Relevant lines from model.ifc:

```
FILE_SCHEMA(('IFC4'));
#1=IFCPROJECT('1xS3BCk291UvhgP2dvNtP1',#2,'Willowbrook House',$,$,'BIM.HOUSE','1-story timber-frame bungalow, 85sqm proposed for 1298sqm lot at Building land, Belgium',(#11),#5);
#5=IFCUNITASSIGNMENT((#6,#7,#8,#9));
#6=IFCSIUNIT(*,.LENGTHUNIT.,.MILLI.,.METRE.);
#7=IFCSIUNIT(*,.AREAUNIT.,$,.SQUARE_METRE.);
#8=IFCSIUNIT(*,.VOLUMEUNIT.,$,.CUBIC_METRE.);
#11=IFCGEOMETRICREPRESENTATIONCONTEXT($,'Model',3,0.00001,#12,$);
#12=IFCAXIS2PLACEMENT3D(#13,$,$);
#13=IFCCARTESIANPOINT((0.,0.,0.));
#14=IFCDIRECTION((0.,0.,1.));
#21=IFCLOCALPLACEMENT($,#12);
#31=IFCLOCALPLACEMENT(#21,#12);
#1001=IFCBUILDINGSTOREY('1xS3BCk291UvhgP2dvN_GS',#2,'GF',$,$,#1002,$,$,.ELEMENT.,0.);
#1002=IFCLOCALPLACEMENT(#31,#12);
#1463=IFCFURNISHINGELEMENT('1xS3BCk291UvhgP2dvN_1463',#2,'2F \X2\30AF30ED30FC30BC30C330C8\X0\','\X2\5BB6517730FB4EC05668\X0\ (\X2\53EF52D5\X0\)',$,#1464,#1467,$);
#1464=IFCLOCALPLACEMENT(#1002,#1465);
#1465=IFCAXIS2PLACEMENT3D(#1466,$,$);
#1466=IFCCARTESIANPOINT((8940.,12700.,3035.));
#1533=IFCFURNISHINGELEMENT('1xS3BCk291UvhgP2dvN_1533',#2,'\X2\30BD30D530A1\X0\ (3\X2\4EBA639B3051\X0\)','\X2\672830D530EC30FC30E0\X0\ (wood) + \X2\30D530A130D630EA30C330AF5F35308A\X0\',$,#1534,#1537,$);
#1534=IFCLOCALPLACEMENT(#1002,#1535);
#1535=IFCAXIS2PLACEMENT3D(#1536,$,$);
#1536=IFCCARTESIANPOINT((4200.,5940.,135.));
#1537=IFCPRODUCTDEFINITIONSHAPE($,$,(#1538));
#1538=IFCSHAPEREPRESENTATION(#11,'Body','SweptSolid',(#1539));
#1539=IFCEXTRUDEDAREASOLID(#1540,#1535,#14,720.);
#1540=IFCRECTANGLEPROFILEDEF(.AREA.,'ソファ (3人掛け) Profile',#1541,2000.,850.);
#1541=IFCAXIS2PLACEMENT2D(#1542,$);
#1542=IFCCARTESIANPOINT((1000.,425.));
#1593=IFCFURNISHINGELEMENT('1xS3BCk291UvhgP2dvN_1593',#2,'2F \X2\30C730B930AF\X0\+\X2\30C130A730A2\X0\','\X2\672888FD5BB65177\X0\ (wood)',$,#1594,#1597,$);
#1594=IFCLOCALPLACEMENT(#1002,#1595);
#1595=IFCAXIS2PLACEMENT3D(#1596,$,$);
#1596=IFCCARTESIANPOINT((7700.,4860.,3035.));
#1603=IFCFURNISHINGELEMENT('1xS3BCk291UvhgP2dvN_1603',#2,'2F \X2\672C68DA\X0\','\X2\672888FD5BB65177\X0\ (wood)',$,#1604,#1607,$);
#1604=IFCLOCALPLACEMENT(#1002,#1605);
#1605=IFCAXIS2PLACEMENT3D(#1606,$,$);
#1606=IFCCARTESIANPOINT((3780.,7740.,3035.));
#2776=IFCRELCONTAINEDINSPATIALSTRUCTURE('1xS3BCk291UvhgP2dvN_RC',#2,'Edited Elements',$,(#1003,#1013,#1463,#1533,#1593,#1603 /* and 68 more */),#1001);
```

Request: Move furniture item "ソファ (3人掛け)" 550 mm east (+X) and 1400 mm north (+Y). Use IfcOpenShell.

```python
import ifcopenshell
import ifcopenshell.api.geometry
import ifcopenshell.util.placement
import ifcopenshell.util.unit

model = ifcopenshell.open("model.ifc")
unit_scale = ifcopenshell.util.unit.calculate_unit_scale(model)

item = model.by_guid("1xS3BCk291UvhgP2dvN_1533")
matrix = ifcopenshell.util.placement.get_local_placement(item.ObjectPlacement)
matrix[0, 3] += 0.55 / unit_scale
matrix[1, 3] += 1.4 / unit_scale
ifcopenshell.api.geometry.edit_object_placement(model, product=item, matrix=matrix, is_si=False)

print(ifcopenshell.util.placement.get_local_placement(item.ObjectPlacement).round(3) + 0.0)

model.write("model_edited.ifc")
```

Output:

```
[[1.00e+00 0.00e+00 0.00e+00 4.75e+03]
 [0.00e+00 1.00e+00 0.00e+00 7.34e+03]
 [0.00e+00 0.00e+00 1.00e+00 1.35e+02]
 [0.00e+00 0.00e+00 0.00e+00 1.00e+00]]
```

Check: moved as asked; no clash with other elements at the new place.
